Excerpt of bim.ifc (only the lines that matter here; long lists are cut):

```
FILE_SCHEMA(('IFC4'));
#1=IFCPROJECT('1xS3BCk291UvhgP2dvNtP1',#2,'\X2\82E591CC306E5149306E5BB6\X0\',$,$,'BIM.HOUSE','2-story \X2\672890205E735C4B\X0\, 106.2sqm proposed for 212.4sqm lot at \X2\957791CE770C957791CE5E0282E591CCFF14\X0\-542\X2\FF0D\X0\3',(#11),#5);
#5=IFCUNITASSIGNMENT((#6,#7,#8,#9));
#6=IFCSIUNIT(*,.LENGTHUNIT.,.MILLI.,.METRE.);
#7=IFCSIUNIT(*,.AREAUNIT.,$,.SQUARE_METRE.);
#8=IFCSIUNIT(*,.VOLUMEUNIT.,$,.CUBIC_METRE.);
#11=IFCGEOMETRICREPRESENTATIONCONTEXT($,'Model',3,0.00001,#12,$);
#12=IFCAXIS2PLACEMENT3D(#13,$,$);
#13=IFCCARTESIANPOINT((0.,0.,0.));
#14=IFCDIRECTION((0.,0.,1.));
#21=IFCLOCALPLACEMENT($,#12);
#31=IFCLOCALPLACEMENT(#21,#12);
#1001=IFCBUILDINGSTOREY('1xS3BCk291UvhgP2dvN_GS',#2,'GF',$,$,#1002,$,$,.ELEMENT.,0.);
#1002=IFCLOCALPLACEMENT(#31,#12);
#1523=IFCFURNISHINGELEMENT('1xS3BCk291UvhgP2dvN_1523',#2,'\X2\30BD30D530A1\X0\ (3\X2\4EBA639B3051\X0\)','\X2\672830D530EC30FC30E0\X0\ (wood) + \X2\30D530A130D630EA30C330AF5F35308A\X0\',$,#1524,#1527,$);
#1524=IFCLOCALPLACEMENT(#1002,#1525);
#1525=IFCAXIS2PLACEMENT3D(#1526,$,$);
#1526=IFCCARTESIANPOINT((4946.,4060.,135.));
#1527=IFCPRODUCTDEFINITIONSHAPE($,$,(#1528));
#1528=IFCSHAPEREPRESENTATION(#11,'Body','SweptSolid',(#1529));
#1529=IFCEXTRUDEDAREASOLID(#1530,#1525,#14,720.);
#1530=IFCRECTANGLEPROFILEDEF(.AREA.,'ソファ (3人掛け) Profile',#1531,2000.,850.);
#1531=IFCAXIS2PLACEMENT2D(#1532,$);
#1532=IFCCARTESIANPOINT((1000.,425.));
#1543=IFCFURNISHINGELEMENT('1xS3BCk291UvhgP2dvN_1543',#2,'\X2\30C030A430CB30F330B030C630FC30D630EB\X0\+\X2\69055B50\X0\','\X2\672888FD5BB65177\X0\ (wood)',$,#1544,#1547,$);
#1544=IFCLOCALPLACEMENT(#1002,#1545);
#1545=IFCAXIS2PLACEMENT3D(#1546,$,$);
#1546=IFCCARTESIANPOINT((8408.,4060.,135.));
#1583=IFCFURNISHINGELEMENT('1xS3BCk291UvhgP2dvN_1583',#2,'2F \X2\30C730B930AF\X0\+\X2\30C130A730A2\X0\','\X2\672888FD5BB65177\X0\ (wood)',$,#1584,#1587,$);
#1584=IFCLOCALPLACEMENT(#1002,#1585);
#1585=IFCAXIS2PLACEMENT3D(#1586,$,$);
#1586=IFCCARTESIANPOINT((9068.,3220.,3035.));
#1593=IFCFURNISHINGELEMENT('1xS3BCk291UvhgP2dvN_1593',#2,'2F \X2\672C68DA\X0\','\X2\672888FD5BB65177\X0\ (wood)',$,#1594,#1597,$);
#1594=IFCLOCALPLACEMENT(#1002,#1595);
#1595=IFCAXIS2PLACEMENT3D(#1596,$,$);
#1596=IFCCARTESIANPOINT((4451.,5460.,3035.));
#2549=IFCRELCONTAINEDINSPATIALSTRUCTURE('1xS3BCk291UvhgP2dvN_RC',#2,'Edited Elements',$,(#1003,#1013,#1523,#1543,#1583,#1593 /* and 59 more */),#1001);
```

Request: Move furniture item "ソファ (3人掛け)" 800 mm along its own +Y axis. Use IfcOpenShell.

```python
import ifcopenshell
import ifcopenshell.api.geometry
import ifcopenshell.util.placement
import ifcopenshell.util.unit

model = ifcopenshell.open("bim.ifc")
unit_scale = ifcopenshell.util.unit.calculate_unit_scale(model)

item = model.by_id(1523)
matrix = ifcopenshell.util.placement.get_local_placement(item.ObjectPlacement)
matrix[:3, 3] += matrix[:3, 1] * 0.8 / unit_scale
ifcopenshell.api.geometry.edit_object_placement(model, product=item, matrix=matrix, is_si=False)

print(ifcopenshell.util.placement.get_local_placement(item.ObjectPlacement).round(3) + 0.0)

model.write("bim_rev.ifc")
```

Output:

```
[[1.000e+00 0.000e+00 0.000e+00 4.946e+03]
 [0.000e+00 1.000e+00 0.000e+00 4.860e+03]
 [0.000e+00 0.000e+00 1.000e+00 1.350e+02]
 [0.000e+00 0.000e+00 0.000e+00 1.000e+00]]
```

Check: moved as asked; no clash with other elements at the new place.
